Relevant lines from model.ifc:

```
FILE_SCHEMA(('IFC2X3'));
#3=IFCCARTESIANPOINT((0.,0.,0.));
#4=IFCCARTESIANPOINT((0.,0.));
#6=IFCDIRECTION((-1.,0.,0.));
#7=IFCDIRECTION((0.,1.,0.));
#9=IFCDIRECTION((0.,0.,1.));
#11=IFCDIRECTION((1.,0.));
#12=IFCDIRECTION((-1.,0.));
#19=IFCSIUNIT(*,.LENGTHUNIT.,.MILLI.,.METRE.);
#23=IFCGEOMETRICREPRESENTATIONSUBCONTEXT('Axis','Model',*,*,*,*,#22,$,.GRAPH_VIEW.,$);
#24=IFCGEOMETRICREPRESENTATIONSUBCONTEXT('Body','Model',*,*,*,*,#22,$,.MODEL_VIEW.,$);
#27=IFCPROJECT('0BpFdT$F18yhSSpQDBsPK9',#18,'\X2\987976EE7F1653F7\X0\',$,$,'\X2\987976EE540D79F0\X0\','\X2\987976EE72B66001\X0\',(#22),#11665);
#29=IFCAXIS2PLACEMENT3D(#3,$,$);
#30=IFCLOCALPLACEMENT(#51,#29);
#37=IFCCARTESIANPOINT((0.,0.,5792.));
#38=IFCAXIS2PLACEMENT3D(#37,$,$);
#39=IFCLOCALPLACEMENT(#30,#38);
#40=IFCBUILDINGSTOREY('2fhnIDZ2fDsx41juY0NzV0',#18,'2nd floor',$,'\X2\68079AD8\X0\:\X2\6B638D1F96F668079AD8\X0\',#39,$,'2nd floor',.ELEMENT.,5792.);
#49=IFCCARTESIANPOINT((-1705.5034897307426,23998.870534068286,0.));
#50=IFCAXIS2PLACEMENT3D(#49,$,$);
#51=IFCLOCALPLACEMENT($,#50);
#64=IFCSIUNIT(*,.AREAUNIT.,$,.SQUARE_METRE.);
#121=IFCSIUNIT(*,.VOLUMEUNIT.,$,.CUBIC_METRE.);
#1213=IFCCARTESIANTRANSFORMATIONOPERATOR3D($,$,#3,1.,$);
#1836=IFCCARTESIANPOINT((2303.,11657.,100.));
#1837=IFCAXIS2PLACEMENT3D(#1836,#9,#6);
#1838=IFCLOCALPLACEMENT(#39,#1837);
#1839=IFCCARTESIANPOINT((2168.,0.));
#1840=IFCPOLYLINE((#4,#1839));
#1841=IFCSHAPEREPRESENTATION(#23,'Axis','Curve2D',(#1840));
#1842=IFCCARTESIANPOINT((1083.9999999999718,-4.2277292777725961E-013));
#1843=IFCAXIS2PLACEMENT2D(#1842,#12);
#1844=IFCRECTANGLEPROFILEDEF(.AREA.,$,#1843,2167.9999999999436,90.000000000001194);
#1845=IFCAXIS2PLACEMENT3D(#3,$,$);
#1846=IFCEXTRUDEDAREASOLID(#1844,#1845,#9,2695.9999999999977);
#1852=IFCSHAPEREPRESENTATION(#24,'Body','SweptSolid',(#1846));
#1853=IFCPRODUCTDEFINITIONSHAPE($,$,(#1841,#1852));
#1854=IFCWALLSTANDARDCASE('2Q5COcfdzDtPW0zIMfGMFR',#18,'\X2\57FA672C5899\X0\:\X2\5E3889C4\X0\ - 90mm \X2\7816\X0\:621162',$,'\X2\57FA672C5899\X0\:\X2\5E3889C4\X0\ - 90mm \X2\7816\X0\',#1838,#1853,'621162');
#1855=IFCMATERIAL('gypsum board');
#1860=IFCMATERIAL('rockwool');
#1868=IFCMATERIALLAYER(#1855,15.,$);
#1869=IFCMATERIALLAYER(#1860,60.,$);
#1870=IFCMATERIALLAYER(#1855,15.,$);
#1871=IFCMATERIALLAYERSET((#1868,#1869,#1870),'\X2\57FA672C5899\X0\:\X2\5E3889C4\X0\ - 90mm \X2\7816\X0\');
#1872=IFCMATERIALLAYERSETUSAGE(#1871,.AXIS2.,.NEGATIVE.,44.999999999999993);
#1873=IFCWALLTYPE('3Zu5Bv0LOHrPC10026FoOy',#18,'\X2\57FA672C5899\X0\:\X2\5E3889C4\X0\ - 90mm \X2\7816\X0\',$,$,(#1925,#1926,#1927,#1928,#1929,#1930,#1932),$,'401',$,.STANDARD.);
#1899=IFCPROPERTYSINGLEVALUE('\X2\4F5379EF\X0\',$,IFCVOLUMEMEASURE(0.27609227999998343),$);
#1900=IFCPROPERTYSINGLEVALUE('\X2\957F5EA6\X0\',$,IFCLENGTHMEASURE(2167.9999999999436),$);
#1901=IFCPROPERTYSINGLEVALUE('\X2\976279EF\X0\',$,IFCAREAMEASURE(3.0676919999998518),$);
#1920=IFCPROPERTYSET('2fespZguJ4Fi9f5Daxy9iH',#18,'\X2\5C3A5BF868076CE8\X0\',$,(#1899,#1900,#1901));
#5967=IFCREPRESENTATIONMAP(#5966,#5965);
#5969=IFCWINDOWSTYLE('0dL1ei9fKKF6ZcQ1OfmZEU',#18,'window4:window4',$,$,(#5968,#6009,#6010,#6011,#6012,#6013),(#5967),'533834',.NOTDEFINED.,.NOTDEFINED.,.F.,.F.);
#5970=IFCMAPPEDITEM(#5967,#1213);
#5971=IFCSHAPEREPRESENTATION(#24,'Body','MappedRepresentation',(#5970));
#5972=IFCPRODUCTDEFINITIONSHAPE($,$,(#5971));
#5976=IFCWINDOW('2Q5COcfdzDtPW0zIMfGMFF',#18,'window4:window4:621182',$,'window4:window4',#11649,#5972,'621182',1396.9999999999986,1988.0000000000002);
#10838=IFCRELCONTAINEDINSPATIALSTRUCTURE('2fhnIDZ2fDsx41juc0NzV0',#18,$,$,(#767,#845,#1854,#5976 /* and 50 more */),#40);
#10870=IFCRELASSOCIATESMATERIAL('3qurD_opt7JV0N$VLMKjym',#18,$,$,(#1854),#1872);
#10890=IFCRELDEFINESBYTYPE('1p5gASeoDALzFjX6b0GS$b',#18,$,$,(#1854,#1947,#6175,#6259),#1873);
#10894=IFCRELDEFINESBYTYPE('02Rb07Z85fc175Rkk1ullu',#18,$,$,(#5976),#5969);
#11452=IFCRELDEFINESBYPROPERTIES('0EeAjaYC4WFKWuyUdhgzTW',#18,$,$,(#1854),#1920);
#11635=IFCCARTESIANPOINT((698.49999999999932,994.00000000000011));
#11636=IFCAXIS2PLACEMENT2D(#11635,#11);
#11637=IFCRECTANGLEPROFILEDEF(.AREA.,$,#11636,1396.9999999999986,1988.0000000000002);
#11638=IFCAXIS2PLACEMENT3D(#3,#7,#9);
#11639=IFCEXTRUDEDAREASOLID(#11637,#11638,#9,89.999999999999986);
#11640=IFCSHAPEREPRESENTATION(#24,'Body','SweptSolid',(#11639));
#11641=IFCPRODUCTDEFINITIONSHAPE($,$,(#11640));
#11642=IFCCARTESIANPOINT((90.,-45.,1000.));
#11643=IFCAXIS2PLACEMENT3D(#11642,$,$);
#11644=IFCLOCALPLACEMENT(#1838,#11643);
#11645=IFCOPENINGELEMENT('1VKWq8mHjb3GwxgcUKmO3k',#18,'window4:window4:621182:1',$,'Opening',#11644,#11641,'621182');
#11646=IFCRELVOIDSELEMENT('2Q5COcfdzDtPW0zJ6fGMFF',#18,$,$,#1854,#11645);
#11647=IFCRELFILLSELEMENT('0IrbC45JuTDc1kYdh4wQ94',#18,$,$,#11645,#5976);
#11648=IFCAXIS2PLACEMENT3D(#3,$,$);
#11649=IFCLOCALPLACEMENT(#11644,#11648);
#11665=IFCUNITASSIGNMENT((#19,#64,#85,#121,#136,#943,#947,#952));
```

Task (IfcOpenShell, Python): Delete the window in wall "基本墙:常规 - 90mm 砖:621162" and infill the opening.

```python
import ifcopenshell
import ifcopenshell.api.feature
import ifcopenshell.api.pset
import ifcopenshell.api.root
import ifcopenshell.geom
import ifcopenshell.util.element
import ifcopenshell.util.shape
import ifcopenshell.util.unit

model = ifcopenshell.open("model.ifc")
area_scale = ifcopenshell.util.unit.calculate_unit_scale(model, "AREAUNIT")
volume_scale = ifcopenshell.util.unit.calculate_unit_scale(model, "VOLUMEUNIT")
settings = ifcopenshell.geom.settings()


def volume(element):
    """Net volume in cubic metres, openings subtracted."""
    shape = ifcopenshell.geom.create_shape(settings, element)
    return ifcopenshell.util.shape.get_volume(shape.geometry)


window = model.by_guid("2Q5COcfdzDtPW0zIMfGMFF")
opening = window.FillsVoids[0].RelatingOpeningElement
wall = opening.VoidsElements[0].RelatingBuildingElement
before = volume(wall)

ifcopenshell.api.root.remove_product(model, product=window)
ifcopenshell.api.feature.remove_feature(model, feature=opening)

after = volume(wall)
thickness = 0.09  # wall thickness in metres

# Update the wall's stored quantities.
pset = model.by_id(ifcopenshell.util.element.get_pset(wall, "尺寸标注", should_inherit=False)["id"])
ifcopenshell.api.pset.edit_pset(model, pset=pset, properties={
    "体积": model.create_entity("IfcVolumeMeasure", after / volume_scale),
    "面积": model.create_entity("IfcAreaMeasure", after / thickness / area_scale),
})

print(f"wall volume {before:.3f} -> {after:.3f} m3")

model.write("model_rev.ifc")
```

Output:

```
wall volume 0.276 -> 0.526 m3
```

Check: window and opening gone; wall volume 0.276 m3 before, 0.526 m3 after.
